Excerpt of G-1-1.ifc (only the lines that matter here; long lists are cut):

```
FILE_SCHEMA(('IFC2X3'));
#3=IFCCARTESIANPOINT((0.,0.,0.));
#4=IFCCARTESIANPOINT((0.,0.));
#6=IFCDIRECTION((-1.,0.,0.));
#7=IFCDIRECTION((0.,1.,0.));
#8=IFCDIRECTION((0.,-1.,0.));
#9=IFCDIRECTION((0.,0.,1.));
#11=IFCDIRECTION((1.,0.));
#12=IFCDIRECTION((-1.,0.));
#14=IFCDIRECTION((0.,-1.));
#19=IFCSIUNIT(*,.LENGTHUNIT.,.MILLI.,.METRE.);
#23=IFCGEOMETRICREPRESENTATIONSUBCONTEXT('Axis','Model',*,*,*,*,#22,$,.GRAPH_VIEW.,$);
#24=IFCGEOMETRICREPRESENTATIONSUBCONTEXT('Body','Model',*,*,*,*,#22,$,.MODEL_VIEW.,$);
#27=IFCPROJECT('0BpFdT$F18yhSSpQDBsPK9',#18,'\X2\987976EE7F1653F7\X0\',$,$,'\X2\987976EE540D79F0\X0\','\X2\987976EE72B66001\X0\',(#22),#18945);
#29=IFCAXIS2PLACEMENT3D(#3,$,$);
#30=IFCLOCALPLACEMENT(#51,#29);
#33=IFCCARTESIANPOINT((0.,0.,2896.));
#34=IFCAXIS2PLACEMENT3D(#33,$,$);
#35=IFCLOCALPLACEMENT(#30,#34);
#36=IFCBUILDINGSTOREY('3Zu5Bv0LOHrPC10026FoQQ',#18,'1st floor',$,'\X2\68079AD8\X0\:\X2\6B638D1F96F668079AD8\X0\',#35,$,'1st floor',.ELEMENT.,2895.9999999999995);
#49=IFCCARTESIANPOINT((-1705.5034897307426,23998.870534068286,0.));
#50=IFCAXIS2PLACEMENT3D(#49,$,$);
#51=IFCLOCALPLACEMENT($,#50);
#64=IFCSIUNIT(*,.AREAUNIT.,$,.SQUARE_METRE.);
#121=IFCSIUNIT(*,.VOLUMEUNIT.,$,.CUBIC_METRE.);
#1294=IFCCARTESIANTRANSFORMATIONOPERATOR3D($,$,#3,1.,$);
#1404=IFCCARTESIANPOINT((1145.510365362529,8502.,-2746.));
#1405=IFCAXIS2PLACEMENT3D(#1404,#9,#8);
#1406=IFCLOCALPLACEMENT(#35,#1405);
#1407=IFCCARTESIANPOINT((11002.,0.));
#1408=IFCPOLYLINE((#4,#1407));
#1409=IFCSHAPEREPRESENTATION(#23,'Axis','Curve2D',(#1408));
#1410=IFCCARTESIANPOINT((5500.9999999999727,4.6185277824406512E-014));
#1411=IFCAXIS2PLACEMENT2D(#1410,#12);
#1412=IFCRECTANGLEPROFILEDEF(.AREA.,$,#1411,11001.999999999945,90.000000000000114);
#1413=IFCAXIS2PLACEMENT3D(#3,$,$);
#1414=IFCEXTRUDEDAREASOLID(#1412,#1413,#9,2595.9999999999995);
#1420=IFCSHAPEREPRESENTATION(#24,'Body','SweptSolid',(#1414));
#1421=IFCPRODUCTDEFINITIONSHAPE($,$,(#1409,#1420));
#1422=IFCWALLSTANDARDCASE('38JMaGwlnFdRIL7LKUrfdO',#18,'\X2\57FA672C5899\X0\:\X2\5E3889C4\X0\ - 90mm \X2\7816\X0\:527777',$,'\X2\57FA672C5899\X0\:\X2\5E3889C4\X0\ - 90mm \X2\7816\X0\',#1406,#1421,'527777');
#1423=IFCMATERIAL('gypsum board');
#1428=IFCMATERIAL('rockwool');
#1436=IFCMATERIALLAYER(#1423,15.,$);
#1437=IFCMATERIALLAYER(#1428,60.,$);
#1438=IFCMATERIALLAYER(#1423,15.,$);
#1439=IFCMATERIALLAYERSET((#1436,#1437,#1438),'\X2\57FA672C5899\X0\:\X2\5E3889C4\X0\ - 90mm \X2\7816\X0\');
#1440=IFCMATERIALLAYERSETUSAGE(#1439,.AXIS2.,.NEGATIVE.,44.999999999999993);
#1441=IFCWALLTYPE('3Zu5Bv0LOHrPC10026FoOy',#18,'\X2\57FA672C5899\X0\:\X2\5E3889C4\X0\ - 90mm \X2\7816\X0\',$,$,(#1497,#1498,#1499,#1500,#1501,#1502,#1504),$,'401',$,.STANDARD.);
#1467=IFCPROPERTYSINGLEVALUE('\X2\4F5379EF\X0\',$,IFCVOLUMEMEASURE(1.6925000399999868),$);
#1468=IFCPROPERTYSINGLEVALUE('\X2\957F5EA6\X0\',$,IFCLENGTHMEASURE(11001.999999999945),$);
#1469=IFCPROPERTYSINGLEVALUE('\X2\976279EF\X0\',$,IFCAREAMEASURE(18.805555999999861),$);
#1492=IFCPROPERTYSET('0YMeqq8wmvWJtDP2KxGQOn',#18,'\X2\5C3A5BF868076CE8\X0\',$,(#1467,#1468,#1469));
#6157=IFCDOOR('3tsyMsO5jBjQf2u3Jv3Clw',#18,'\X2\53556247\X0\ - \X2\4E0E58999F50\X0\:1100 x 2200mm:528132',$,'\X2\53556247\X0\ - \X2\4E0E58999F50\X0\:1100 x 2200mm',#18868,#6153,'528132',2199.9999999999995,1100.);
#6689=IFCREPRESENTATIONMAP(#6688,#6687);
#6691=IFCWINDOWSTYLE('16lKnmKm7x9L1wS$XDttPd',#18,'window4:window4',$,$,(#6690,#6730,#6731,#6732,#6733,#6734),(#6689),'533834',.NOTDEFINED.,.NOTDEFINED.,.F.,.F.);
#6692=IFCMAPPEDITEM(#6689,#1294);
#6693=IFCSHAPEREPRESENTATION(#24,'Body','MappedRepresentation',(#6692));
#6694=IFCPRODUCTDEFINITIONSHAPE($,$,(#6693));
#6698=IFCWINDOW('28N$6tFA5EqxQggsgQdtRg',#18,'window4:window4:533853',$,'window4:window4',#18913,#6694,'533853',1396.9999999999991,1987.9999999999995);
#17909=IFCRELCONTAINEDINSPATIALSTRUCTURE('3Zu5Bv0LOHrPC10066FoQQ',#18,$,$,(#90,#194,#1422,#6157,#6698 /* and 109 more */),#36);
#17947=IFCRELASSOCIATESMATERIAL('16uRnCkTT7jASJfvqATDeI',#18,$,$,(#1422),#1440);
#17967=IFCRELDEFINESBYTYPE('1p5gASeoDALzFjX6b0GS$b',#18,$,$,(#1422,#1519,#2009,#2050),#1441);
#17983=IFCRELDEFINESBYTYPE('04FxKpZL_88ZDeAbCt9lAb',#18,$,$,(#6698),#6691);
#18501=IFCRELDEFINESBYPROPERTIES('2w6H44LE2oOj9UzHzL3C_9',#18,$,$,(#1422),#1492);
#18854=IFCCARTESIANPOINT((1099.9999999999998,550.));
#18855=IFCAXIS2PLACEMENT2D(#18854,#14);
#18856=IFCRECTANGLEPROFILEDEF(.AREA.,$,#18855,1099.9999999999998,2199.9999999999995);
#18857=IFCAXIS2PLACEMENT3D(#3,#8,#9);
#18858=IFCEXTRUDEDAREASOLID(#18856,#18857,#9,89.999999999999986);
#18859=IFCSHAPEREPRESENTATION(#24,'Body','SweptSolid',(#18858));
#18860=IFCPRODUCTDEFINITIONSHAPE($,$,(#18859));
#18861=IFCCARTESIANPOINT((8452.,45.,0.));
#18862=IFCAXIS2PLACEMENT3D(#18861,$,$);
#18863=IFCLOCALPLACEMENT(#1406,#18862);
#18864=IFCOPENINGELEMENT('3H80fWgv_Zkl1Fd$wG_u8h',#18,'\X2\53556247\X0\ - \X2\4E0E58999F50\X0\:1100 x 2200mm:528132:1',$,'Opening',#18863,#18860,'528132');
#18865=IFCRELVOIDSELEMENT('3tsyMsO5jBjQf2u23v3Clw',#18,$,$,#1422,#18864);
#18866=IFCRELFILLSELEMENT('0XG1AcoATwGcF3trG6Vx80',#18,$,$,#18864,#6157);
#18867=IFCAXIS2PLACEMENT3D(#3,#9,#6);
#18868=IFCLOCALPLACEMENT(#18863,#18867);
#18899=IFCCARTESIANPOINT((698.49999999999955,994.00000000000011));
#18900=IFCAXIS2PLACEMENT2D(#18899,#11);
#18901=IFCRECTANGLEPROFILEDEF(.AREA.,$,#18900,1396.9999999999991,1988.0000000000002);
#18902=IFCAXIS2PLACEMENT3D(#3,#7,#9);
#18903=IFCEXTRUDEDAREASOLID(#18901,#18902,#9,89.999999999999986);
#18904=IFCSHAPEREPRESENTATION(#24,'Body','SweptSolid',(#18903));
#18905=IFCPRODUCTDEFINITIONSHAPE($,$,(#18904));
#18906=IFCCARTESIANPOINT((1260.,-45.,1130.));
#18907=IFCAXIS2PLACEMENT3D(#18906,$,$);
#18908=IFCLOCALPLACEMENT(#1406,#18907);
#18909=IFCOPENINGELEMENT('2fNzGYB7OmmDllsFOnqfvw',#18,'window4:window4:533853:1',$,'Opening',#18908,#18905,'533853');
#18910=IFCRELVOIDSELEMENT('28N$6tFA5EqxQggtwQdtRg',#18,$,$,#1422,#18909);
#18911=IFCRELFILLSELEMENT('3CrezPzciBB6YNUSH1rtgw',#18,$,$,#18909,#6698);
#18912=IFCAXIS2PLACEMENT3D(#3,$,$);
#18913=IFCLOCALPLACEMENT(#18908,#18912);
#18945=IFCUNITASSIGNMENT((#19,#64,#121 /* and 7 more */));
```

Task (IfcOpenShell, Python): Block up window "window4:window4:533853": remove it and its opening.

```python
import ifcopenshell
import ifcopenshell.api.feature
import ifcopenshell.api.pset
import ifcopenshell.api.root
import ifcopenshell.geom
import ifcopenshell.util.element
import ifcopenshell.util.shape
import ifcopenshell.util.unit

model = ifcopenshell.open("G-1-1.ifc")
area_scale = ifcopenshell.util.unit.calculate_unit_scale(model, "AREAUNIT")
volume_scale = ifcopenshell.util.unit.calculate_unit_scale(model, "VOLUMEUNIT")
settings = ifcopenshell.geom.settings()


def volume(element):
    """Net volume in cubic metres, openings subtracted."""
    shape = ifcopenshell.geom.create_shape(settings, element)
    return ifcopenshell.util.shape.get_volume(shape.geometry)


window = model.by_guid("28N$6tFA5EqxQggsgQdtRg")
opening = window.FillsVoids[0].RelatingOpeningElement
wall = opening.VoidsElements[0].RelatingBuildingElement
before = volume(wall)

ifcopenshell.api.root.remove_product(model, product=window)
ifcopenshell.api.feature.remove_feature(model, feature=opening)

after = volume(wall)
thickness = 0.09  # wall thickness in metres

# Update the wall's stored quantities.
pset = model.by_id(ifcopenshell.util.element.get_pset(wall, "尺寸标注", should_inherit=False)["id"])
ifcopenshell.api.pset.edit_pset(model, pset=pset, properties={
    "体积": model.create_entity("IfcVolumeMeasure", after / volume_scale),
    "面积": model.create_entity("IfcAreaMeasure", after / thickness / area_scale),
})

print(f"wall volume {before:.3f} -> {after:.3f} m3")

model.write("G-1-1_rev.ifc")
```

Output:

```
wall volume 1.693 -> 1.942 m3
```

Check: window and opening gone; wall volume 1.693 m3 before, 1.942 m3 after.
